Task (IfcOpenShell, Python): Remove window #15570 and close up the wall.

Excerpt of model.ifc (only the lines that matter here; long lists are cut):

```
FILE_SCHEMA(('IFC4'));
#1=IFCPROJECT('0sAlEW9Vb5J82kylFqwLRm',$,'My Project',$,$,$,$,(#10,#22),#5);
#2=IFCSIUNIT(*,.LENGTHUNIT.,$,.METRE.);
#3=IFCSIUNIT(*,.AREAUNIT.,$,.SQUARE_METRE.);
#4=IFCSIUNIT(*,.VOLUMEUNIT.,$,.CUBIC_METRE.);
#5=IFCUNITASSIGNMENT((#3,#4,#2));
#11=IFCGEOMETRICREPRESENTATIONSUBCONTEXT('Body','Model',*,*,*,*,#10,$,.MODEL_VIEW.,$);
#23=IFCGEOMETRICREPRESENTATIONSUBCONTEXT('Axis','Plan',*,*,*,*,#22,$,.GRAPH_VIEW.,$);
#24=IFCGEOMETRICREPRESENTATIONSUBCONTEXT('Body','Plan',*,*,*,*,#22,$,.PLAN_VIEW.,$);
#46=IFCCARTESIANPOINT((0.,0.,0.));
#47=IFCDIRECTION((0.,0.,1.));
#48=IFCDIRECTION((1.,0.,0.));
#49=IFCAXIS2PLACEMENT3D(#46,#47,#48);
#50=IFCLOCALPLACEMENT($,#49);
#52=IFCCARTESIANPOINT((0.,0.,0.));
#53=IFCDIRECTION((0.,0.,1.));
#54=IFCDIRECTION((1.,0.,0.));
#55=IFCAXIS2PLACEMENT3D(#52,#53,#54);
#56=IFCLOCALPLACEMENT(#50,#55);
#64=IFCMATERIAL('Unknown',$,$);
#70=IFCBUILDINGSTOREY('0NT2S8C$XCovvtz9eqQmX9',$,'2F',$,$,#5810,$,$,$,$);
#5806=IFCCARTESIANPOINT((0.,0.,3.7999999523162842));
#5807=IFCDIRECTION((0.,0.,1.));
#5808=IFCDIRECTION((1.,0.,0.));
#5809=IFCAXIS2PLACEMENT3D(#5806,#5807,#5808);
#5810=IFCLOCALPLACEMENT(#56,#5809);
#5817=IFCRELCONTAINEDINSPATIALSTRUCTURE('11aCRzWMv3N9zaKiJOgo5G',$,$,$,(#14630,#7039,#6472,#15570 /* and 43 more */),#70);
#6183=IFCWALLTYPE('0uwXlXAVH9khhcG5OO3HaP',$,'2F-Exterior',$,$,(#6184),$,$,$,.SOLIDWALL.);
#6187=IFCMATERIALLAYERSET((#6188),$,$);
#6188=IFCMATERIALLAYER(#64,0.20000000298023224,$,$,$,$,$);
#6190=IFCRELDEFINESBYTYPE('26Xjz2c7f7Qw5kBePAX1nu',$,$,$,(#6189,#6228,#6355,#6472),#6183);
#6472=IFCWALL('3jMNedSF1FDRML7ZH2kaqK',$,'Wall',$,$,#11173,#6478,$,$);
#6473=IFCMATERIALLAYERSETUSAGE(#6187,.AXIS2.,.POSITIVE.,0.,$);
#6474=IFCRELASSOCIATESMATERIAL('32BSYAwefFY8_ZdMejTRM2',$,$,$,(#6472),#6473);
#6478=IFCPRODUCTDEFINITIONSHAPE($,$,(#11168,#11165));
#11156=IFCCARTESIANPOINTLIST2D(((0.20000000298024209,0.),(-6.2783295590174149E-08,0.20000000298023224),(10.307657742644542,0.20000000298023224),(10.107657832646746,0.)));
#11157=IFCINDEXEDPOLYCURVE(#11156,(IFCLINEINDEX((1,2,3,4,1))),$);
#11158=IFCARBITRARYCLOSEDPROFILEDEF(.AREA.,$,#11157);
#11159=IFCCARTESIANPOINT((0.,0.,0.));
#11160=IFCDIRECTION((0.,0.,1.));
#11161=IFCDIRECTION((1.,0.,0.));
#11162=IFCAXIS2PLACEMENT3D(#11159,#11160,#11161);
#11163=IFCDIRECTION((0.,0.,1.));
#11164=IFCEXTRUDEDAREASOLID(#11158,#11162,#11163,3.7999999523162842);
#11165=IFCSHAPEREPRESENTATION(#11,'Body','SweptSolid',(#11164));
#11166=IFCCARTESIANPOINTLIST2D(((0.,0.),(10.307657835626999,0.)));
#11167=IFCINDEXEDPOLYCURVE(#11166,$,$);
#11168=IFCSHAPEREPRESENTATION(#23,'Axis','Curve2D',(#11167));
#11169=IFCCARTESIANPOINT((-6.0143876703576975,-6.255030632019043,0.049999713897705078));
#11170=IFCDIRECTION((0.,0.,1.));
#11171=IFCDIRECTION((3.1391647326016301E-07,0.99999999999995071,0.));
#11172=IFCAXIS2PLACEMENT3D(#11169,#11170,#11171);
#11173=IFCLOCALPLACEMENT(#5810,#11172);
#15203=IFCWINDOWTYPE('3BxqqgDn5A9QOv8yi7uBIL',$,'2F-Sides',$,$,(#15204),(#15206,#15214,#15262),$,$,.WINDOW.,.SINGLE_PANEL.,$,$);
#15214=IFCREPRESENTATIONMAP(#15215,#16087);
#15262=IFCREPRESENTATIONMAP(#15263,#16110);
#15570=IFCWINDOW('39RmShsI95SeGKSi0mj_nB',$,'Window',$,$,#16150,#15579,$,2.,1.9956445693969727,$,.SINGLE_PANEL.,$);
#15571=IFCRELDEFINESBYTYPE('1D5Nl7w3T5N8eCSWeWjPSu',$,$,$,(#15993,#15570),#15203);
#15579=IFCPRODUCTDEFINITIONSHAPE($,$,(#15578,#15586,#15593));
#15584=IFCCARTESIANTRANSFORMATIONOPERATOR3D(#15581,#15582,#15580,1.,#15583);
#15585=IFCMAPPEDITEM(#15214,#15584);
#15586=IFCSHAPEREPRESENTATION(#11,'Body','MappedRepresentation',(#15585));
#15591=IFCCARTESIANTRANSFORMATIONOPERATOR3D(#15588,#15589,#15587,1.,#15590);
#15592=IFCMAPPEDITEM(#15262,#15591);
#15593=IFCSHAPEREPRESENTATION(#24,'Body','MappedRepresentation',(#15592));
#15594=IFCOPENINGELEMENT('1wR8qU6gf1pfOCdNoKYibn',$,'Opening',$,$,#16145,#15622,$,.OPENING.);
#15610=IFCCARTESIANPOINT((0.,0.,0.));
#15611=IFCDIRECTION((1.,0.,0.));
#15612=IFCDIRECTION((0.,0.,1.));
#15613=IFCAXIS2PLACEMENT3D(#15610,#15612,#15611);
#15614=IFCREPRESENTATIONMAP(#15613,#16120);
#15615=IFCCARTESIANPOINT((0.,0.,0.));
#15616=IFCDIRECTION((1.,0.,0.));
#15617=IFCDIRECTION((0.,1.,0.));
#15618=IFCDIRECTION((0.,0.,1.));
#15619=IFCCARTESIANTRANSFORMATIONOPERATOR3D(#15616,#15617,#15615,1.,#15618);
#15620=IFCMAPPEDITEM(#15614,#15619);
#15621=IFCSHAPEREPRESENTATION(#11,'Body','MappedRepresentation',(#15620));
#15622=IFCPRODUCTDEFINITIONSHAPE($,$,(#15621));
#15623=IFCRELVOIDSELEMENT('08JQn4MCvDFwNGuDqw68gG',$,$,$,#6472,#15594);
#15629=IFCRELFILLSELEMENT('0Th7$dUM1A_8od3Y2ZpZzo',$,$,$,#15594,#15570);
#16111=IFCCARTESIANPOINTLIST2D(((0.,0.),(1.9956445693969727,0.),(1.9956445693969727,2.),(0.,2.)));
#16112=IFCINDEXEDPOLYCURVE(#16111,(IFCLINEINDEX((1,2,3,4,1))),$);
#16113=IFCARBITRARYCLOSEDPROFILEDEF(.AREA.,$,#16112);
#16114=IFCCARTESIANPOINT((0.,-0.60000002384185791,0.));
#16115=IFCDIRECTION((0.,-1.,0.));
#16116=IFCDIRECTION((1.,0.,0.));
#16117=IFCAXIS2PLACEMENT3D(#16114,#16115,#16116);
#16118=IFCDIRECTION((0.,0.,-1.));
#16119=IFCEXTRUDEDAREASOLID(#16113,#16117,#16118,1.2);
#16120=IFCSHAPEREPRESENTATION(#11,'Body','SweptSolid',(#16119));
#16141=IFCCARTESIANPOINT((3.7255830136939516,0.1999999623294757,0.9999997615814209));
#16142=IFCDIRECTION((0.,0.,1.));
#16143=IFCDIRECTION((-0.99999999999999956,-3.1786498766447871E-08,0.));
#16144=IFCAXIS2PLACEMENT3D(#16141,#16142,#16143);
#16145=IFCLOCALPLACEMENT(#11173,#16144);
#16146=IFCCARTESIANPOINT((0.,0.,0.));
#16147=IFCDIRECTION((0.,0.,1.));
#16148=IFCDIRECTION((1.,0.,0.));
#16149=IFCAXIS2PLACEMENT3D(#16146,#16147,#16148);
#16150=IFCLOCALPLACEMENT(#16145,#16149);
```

```python
import ifcopenshell
import ifcopenshell.api.feature
import ifcopenshell.api.root
import ifcopenshell.geom
import ifcopenshell.util.shape

model = ifcopenshell.open("model.ifc")
settings = ifcopenshell.geom.settings()


def volume(element):
    """Net volume in cubic metres, openings subtracted."""
    shape = ifcopenshell.geom.create_shape(settings, element)
    return ifcopenshell.util.shape.get_volume(shape.geometry)


window = model.by_guid("39RmShsI95SeGKSi0mj_nB")
opening = window.FillsVoids[0].RelatingOpeningElement
wall = opening.VoidsElements[0].RelatingBuildingElement
before = volume(wall)

ifcopenshell.api.root.remove_product(model, product=window)
ifcopenshell.api.feature.remove_feature(model, feature=opening)

after = volume(wall)

print(f"wall volume {before:.3f} -> {after:.3f} m3")

model.write("model_v2.ifc")
```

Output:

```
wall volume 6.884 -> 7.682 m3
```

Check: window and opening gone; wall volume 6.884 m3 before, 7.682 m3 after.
